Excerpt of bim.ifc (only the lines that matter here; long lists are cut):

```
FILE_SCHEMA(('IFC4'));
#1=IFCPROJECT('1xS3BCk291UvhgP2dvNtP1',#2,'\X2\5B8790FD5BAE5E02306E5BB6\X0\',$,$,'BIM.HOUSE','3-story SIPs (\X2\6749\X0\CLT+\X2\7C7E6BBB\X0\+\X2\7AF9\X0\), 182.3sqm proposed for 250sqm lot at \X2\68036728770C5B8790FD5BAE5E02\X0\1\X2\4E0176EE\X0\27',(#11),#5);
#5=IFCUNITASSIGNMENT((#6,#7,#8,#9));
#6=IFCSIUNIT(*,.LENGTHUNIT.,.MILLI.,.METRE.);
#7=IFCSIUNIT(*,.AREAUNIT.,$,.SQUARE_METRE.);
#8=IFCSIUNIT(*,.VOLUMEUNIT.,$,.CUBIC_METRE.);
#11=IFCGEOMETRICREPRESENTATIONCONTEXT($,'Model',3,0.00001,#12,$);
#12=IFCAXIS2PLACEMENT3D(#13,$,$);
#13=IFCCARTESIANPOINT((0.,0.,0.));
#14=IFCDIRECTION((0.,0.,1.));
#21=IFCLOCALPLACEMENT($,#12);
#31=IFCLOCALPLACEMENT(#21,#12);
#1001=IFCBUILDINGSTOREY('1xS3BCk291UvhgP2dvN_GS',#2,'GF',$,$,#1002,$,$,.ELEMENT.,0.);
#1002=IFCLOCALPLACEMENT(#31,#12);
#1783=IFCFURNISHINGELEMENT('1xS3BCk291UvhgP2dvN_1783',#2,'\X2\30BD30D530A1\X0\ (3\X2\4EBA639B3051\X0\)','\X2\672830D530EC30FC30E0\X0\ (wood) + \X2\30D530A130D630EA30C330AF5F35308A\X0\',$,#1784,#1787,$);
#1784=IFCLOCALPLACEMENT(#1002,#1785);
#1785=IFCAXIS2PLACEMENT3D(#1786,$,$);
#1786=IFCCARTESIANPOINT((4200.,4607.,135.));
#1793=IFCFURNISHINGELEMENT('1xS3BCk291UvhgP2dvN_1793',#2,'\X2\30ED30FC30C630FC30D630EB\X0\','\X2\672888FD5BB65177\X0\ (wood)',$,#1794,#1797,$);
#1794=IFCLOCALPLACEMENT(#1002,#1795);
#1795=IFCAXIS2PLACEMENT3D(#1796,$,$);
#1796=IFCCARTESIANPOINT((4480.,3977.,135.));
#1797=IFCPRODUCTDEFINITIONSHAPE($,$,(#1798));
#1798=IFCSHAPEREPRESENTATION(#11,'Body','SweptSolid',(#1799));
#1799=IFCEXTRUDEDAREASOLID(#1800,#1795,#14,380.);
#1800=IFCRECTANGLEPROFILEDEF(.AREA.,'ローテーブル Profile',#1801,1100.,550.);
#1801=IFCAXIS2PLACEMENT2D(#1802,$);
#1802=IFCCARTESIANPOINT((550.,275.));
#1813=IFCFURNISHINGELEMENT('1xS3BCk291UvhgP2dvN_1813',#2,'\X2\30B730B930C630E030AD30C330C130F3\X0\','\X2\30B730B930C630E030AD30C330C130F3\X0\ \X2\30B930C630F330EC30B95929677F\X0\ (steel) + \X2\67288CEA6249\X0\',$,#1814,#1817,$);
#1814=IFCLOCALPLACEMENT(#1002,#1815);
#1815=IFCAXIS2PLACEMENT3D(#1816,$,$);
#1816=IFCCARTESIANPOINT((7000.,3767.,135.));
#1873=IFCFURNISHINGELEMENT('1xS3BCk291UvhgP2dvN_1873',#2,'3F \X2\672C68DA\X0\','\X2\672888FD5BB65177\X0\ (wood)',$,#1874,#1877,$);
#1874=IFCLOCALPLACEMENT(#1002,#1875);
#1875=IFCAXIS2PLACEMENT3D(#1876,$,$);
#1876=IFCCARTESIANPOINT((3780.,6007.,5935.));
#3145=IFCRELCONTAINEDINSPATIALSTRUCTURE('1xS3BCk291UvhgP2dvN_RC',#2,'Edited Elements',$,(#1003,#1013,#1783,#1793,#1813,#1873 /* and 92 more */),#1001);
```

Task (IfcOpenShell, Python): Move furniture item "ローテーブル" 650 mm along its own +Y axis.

```python
import ifcopenshell
import ifcopenshell.api.geometry
import ifcopenshell.util.placement

model = ifcopenshell.open("bim.ifc")

item = model.by_guid("1xS3BCk291UvhgP2dvN_1793")
matrix = ifcopenshell.util.placement.get_local_placement(item.ObjectPlacement)
matrix[:3, 3] += matrix[:3, 1] * 650.0
ifcopenshell.api.geometry.edit_object_placement(model, product=item, matrix=matrix, is_si=False)

print(ifcopenshell.util.placement.get_local_placement(item.ObjectPlacement).round(3) + 0.0)

model.write("bim-out.ifc")
```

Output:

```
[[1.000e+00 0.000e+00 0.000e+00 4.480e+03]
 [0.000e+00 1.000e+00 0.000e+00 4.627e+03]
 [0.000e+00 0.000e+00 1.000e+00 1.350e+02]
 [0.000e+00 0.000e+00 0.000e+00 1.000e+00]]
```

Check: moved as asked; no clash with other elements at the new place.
